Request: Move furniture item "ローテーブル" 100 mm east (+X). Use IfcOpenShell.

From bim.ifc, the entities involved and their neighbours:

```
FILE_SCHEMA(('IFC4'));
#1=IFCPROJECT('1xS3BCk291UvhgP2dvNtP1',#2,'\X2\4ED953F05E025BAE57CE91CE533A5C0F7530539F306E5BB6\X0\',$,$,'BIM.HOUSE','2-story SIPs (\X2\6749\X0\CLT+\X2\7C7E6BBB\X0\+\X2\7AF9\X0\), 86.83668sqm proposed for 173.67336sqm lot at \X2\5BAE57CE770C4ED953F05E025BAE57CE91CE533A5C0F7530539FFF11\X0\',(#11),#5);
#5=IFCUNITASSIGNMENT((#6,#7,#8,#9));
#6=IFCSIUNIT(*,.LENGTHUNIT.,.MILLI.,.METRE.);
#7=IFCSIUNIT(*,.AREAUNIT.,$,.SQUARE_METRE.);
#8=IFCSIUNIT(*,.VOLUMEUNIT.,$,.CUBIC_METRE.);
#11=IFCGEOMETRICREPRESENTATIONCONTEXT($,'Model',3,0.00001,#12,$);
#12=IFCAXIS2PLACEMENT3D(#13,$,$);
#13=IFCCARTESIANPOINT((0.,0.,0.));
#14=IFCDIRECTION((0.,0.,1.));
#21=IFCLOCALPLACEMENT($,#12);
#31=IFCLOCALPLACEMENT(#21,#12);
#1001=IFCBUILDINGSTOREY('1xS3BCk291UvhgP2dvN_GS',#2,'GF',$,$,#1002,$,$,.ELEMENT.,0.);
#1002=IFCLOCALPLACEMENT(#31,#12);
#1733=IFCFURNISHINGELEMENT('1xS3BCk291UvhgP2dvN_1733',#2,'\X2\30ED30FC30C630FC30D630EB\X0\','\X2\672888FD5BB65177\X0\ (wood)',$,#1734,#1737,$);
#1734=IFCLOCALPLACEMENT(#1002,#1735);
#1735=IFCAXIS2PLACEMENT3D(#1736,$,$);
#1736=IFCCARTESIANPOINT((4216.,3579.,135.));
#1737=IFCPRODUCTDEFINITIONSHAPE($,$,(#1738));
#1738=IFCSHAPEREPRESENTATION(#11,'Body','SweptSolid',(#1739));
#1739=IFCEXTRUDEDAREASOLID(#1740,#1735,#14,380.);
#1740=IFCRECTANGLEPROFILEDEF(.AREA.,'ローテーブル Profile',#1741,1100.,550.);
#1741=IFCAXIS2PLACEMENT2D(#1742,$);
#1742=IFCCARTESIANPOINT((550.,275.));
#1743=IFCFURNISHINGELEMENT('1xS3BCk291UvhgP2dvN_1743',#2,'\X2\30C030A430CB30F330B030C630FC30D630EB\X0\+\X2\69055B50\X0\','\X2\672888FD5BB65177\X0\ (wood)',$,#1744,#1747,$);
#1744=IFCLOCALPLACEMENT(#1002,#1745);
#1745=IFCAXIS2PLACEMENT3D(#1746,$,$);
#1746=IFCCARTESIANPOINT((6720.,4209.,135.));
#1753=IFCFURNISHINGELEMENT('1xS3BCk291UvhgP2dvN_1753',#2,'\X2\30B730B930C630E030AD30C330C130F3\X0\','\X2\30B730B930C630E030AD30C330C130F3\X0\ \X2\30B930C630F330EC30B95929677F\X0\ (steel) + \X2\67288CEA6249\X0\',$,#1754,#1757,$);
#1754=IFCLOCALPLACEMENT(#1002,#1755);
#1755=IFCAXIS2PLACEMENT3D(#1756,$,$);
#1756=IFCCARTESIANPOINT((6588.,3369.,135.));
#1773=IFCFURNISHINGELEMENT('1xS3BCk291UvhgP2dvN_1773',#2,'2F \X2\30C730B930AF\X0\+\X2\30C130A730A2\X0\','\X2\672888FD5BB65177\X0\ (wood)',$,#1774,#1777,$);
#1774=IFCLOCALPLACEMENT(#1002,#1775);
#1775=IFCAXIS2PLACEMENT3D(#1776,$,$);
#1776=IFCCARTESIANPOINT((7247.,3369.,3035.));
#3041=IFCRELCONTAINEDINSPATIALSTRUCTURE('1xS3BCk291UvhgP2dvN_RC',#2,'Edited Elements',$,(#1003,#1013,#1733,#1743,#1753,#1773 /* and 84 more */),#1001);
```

```python
import ifcopenshell
import ifcopenshell.api.geometry
import ifcopenshell.util.placement
import ifcopenshell.util.unit

model = ifcopenshell.open("bim.ifc")
unit_scale = ifcopenshell.util.unit.calculate_unit_scale(model)

item = model.by_id(1733)
matrix = ifcopenshell.util.placement.get_local_placement(item.ObjectPlacement)
matrix[0, 3] += 0.1 / unit_scale
ifcopenshell.api.geometry.edit_object_placement(model, product=item, matrix=matrix, is_si=False)

print(ifcopenshell.util.placement.get_local_placement(item.ObjectPlacement).round(3) + 0.0)

model.write("bim_edited.ifc")
```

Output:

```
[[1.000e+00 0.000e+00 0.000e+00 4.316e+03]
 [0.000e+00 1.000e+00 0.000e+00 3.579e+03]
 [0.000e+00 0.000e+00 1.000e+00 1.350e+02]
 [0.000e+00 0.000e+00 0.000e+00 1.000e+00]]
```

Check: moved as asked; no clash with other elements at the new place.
